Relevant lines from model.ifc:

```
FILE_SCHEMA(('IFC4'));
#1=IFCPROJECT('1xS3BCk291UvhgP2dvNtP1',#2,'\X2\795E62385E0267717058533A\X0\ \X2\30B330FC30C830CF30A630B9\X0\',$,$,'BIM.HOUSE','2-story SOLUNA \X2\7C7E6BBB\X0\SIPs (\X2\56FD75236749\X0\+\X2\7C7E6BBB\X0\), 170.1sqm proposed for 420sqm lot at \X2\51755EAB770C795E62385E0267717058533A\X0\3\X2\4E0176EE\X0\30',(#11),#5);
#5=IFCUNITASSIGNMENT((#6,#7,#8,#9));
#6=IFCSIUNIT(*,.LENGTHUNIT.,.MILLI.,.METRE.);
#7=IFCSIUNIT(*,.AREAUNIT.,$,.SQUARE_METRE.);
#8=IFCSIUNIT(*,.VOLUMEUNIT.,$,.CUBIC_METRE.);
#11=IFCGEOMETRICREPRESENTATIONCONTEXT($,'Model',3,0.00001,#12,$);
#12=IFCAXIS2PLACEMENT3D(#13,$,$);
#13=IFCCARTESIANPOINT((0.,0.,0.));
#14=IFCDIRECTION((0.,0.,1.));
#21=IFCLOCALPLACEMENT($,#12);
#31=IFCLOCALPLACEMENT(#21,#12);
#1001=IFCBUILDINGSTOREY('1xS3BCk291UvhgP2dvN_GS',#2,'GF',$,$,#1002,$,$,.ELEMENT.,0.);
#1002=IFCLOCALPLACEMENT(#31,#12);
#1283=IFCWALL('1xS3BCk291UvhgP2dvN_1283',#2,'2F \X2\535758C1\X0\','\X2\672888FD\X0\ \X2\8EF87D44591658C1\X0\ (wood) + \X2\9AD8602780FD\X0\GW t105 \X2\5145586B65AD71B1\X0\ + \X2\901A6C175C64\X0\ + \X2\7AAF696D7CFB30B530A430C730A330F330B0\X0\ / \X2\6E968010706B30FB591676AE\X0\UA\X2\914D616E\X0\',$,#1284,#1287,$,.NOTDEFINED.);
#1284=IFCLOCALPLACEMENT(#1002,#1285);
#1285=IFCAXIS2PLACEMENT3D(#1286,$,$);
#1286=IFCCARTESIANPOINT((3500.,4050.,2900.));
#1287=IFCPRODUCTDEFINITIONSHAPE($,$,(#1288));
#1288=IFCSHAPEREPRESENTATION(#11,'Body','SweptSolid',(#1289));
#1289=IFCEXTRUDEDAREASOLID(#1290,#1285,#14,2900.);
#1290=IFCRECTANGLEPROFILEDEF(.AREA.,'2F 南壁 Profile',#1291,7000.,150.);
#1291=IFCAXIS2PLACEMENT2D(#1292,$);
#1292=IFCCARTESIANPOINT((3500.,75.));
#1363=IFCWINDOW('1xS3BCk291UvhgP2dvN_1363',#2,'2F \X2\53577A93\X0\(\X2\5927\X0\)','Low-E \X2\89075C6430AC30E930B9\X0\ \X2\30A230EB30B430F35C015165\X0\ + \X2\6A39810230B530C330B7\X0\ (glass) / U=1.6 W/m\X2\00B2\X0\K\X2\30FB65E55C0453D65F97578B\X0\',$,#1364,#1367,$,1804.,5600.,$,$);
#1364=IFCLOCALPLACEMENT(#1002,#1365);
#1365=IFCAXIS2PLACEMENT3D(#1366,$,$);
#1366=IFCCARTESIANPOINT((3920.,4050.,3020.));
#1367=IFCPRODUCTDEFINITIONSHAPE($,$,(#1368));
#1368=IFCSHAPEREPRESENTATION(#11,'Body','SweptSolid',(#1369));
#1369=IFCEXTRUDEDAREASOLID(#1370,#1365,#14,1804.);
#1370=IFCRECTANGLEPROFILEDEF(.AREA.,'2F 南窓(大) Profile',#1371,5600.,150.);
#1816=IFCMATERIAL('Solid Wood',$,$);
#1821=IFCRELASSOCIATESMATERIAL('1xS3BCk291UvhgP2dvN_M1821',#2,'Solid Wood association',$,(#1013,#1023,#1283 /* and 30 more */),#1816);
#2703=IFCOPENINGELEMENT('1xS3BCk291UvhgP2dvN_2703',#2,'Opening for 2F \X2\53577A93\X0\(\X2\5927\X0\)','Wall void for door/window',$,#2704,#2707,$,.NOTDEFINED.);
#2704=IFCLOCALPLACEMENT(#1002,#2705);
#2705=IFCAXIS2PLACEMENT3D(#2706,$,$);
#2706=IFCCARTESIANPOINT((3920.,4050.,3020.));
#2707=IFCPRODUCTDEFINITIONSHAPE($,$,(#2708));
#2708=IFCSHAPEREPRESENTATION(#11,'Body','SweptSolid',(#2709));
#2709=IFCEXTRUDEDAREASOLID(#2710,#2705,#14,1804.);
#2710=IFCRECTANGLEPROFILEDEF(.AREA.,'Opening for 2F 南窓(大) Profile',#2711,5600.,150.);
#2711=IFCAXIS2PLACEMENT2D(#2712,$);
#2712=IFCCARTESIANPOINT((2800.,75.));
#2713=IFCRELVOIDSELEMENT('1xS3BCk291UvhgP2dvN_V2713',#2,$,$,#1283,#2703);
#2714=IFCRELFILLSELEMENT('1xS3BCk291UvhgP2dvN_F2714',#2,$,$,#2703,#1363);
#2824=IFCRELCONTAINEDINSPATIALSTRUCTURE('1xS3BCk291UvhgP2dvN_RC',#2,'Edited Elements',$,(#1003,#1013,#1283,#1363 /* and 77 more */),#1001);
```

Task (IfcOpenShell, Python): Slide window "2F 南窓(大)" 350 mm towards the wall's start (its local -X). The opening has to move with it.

```python
import ifcopenshell
import ifcopenshell.api.geometry
import ifcopenshell.util.placement
import ifcopenshell.util.unit

model = ifcopenshell.open("model.ifc")
unit_scale = ifcopenshell.util.unit.calculate_unit_scale(model)

window = model.by_guid("1xS3BCk291UvhgP2dvN_1363")
opening = window.FillsVoids[0].RelatingOpeningElement
wall = opening.VoidsElements[0].RelatingBuildingElement

wall_matrix = ifcopenshell.util.placement.get_local_placement(wall.ObjectPlacement)
shift = wall_matrix[:3, 0] * -0.35 / unit_scale
before = ifcopenshell.util.placement.get_local_placement(window.ObjectPlacement)[:3, 3].copy()

# The window is not placed relative to its opening, so move both.
for product in (opening, window):
    matrix = ifcopenshell.util.placement.get_local_placement(product.ObjectPlacement)
    matrix[:3, 3] += shift
    ifcopenshell.api.geometry.edit_object_placement(model, product=product, matrix=matrix, is_si=False)

after = ifcopenshell.util.placement.get_local_placement(window.ObjectPlacement)[:3, 3]
print("window moved by", (after - before).round(3) + 0.0)

model.write("model-out.ifc")
```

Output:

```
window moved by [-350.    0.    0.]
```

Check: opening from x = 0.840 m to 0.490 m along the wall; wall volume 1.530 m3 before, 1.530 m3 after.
